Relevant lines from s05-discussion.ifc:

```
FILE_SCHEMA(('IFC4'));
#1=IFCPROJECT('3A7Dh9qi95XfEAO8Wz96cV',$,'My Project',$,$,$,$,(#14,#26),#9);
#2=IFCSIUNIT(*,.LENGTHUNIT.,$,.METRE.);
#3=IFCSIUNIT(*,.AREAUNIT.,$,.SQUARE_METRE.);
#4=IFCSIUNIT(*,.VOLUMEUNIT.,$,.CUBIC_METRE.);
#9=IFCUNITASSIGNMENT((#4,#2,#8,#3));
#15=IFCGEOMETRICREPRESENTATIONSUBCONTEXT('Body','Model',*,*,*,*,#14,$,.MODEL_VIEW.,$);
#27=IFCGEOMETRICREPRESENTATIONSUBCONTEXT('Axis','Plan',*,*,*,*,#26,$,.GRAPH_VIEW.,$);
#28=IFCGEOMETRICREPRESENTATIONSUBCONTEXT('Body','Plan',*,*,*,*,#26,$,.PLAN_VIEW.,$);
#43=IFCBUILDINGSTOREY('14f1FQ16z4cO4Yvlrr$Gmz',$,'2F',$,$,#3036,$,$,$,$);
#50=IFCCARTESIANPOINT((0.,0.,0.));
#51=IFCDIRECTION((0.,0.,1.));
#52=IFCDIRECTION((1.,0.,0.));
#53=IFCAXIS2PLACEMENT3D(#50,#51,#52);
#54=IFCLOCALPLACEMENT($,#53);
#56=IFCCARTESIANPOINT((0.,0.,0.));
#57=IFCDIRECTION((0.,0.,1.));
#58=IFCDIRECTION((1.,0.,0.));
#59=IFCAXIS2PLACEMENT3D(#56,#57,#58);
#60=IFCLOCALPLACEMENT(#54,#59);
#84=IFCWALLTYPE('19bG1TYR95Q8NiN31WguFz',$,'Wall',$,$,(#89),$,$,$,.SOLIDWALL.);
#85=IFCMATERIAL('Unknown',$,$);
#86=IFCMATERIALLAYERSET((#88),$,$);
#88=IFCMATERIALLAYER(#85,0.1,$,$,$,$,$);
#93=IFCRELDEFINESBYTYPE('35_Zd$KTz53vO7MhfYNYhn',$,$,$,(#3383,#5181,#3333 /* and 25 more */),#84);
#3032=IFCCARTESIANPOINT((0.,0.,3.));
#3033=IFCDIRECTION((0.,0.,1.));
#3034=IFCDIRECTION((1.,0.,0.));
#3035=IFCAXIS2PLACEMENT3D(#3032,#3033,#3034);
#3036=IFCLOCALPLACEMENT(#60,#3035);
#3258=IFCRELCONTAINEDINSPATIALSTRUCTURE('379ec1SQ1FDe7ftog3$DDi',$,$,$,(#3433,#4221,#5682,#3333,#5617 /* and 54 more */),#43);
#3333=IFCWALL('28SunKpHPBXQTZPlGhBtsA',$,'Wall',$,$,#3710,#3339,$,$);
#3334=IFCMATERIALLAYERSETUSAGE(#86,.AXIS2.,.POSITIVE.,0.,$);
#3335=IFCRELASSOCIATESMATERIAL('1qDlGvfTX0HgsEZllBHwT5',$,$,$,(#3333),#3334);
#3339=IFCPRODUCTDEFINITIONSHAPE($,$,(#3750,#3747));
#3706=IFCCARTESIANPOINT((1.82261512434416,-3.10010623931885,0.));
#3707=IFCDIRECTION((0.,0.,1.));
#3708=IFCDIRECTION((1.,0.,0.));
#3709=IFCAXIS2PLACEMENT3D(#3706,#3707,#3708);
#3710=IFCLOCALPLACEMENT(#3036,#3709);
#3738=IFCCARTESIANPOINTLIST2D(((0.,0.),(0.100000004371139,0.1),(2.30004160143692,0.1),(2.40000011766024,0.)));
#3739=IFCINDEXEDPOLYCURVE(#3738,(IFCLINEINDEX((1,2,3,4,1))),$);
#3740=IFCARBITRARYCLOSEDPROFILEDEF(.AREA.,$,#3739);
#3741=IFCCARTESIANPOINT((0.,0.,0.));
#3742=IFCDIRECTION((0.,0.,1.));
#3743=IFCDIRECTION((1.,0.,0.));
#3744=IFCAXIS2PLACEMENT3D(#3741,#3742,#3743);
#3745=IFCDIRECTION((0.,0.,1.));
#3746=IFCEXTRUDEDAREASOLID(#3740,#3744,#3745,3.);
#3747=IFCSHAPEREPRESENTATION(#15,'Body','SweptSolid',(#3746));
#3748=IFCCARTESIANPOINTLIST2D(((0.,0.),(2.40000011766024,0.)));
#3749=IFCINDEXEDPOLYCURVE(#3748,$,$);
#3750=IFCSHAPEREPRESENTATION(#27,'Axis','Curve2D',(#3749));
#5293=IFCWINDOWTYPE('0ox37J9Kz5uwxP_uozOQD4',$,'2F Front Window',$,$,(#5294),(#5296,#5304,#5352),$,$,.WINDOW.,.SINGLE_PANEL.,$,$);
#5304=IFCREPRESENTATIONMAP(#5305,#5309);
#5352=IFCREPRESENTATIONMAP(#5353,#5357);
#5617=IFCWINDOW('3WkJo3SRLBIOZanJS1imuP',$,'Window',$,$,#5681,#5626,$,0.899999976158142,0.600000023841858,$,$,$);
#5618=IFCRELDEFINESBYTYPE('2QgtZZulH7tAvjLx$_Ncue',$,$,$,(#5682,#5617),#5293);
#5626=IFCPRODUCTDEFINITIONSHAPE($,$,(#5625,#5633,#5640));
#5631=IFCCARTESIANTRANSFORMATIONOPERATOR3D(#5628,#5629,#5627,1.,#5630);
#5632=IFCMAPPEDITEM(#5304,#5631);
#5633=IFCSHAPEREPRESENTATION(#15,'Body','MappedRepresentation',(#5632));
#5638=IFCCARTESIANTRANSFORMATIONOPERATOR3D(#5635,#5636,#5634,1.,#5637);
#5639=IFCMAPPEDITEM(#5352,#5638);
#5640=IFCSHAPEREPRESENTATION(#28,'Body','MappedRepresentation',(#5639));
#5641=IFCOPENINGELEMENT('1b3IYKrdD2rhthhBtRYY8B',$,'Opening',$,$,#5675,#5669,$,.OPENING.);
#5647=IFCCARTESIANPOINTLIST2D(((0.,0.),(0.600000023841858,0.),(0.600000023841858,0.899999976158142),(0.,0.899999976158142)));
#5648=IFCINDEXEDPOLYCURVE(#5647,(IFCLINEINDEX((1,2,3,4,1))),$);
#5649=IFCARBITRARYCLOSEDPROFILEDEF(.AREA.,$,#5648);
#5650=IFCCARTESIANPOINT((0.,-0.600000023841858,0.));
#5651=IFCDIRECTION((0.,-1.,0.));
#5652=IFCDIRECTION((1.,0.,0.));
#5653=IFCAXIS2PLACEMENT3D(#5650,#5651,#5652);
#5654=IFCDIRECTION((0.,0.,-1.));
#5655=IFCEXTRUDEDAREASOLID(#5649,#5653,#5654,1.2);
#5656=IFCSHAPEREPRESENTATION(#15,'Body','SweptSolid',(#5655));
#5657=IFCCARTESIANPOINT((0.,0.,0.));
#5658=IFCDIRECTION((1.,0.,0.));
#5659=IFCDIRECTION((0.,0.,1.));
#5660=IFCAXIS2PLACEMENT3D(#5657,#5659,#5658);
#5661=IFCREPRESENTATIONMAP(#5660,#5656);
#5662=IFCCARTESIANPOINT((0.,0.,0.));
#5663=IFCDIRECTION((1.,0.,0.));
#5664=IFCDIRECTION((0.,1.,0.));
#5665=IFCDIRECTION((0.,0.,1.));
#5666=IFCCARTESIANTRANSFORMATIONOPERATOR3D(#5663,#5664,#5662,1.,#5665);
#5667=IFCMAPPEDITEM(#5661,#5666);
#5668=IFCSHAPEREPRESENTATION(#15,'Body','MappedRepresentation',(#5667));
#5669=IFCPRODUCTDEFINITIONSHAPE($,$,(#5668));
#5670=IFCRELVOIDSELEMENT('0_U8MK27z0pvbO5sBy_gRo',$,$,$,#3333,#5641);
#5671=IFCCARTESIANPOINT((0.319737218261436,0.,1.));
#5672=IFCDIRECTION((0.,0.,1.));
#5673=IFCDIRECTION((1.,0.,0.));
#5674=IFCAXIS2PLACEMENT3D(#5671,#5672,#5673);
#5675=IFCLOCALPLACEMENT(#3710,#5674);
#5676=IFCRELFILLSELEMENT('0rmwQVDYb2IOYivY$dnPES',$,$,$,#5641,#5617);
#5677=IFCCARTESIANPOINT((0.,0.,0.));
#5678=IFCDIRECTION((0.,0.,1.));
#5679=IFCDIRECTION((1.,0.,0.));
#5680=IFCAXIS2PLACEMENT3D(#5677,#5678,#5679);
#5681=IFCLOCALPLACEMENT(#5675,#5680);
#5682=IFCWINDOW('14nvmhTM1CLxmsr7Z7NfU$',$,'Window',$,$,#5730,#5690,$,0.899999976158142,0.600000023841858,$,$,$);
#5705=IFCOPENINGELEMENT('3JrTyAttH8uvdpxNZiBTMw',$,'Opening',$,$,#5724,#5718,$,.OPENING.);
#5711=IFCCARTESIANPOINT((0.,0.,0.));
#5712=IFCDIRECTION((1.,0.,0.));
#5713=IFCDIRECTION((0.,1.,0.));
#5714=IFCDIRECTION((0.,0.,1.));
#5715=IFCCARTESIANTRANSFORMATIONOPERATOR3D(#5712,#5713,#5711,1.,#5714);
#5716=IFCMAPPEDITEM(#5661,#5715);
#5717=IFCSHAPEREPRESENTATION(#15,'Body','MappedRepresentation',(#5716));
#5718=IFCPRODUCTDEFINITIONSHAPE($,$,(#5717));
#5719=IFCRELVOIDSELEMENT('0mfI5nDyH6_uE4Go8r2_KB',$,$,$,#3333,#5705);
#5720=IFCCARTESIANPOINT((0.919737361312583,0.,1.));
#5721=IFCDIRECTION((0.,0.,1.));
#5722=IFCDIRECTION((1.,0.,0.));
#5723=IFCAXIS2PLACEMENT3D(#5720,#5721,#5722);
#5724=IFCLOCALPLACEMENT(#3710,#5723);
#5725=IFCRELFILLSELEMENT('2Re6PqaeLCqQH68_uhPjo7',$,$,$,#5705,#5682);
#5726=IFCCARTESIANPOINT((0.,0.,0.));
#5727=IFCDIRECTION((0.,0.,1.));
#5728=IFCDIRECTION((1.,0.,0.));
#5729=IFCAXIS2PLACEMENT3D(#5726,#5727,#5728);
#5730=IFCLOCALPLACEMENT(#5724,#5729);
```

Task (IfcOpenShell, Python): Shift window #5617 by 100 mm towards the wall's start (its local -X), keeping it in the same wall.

```python
import ifcopenshell
import ifcopenshell.api.geometry
import ifcopenshell.util.placement

model = ifcopenshell.open("s05-discussion.ifc")

window = model.by_guid("3WkJo3SRLBIOZanJS1imuP")
opening = window.FillsVoids[0].RelatingOpeningElement
wall = opening.VoidsElements[0].RelatingBuildingElement

wall_matrix = ifcopenshell.util.placement.get_local_placement(wall.ObjectPlacement)
shift = wall_matrix[:3, 0] * -0.1
before = ifcopenshell.util.placement.get_local_placement(window.ObjectPlacement)[:3, 3].copy()

# The window is placed relative to its opening, so it follows when the opening moves.
matrix = ifcopenshell.util.placement.get_local_placement(opening.ObjectPlacement)
matrix[:3, 3] += shift
ifcopenshell.api.geometry.edit_object_placement(
    model, product=opening, matrix=matrix, is_si=False, should_transform_children=True
)

after = ifcopenshell.util.placement.get_local_placement(window.ObjectPlacement)[:3, 3]
print("window moved by", (after - before).round(3) + 0.0)

model.write("s05-discussion_v2.ifc")
```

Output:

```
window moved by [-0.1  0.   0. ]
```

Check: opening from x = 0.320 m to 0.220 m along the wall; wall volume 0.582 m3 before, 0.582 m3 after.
